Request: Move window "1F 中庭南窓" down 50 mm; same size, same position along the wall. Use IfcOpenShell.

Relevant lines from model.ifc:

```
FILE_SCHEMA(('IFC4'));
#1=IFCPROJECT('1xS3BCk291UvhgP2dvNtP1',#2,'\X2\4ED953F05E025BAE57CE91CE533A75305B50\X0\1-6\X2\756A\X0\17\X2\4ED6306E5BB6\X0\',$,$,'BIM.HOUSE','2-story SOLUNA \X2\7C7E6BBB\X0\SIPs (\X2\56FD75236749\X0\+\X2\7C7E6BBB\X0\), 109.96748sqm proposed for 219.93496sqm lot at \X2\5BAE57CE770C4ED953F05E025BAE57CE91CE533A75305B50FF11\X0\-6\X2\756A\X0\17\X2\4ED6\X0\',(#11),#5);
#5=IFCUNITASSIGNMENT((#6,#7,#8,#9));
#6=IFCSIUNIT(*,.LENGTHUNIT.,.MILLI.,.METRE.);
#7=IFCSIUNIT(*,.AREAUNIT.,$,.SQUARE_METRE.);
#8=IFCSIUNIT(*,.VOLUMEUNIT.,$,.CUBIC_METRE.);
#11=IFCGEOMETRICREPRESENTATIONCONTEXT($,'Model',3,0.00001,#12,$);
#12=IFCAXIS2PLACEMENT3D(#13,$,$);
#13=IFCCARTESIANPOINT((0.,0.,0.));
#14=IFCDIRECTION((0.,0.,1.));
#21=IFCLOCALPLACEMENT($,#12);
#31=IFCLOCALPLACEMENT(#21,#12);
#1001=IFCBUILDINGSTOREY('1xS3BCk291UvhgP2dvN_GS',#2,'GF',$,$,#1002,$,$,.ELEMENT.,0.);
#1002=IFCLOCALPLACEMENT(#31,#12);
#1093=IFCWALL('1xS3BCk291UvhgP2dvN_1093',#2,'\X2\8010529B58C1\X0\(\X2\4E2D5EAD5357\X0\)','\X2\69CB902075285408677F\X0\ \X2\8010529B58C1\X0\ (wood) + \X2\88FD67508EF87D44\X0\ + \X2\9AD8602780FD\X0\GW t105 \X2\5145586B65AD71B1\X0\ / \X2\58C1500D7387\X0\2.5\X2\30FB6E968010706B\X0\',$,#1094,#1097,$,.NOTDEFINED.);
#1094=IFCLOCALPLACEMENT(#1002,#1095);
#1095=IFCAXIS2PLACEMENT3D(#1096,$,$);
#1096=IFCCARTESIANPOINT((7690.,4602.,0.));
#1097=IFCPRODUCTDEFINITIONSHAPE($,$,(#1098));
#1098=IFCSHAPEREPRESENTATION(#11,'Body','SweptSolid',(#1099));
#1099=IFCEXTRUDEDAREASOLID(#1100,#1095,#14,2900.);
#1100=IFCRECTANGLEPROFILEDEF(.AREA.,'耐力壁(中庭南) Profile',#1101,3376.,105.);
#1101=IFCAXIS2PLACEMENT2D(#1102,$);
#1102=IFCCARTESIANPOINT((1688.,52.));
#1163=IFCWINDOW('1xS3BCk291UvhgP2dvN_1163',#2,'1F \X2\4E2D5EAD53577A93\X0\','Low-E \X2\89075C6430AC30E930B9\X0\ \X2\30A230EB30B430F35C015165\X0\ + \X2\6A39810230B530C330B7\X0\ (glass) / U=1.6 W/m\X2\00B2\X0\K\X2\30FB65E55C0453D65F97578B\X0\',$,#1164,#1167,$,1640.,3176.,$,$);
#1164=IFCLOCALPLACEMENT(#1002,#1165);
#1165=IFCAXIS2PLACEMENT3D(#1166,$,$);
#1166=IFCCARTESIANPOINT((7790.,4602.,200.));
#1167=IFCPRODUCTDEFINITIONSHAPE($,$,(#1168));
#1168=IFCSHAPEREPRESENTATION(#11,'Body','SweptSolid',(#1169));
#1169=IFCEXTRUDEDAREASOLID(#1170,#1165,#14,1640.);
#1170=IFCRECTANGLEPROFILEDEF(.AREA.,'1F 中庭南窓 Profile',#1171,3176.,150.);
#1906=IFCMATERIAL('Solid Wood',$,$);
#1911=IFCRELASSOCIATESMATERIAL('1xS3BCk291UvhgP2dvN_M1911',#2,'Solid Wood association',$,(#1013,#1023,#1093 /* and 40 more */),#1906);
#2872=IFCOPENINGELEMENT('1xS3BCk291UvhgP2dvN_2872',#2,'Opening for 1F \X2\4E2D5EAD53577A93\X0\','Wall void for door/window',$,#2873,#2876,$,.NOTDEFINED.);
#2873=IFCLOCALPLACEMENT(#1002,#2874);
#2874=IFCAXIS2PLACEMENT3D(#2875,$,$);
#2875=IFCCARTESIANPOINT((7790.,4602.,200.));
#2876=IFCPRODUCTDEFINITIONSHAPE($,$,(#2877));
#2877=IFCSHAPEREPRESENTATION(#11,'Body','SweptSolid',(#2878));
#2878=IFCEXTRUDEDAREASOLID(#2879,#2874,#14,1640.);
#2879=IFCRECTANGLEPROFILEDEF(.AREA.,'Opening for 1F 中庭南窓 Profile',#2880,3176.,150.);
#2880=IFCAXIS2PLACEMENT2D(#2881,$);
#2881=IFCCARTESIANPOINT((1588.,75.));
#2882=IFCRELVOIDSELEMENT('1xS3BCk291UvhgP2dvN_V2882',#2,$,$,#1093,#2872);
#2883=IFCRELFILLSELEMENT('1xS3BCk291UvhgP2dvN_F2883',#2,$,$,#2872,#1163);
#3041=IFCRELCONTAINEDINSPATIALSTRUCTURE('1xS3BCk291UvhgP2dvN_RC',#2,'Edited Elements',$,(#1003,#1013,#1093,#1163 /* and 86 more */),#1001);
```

```python
import numpy as np
import ifcopenshell
import ifcopenshell.api.geometry
import ifcopenshell.util.placement
import ifcopenshell.util.unit

model = ifcopenshell.open("model.ifc")
unit_scale = ifcopenshell.util.unit.calculate_unit_scale(model)

window = model.by_guid("1xS3BCk291UvhgP2dvN_1163")
opening = window.FillsVoids[0].RelatingOpeningElement
dz = -50.0

shift = np.array([0.0, 0.0, dz])
# The window is not placed relative to its opening, so move both.
for product in (opening, window):
    matrix = ifcopenshell.util.placement.get_local_placement(product.ObjectPlacement)
    matrix[:3, 3] += shift
    ifcopenshell.api.geometry.edit_object_placement(model, product=product, matrix=matrix, is_si=False)

print(f"moved by {dz * unit_scale:+.3f} m")

model.write("model_rev.ifc")
```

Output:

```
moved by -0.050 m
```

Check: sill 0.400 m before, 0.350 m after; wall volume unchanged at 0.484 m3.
